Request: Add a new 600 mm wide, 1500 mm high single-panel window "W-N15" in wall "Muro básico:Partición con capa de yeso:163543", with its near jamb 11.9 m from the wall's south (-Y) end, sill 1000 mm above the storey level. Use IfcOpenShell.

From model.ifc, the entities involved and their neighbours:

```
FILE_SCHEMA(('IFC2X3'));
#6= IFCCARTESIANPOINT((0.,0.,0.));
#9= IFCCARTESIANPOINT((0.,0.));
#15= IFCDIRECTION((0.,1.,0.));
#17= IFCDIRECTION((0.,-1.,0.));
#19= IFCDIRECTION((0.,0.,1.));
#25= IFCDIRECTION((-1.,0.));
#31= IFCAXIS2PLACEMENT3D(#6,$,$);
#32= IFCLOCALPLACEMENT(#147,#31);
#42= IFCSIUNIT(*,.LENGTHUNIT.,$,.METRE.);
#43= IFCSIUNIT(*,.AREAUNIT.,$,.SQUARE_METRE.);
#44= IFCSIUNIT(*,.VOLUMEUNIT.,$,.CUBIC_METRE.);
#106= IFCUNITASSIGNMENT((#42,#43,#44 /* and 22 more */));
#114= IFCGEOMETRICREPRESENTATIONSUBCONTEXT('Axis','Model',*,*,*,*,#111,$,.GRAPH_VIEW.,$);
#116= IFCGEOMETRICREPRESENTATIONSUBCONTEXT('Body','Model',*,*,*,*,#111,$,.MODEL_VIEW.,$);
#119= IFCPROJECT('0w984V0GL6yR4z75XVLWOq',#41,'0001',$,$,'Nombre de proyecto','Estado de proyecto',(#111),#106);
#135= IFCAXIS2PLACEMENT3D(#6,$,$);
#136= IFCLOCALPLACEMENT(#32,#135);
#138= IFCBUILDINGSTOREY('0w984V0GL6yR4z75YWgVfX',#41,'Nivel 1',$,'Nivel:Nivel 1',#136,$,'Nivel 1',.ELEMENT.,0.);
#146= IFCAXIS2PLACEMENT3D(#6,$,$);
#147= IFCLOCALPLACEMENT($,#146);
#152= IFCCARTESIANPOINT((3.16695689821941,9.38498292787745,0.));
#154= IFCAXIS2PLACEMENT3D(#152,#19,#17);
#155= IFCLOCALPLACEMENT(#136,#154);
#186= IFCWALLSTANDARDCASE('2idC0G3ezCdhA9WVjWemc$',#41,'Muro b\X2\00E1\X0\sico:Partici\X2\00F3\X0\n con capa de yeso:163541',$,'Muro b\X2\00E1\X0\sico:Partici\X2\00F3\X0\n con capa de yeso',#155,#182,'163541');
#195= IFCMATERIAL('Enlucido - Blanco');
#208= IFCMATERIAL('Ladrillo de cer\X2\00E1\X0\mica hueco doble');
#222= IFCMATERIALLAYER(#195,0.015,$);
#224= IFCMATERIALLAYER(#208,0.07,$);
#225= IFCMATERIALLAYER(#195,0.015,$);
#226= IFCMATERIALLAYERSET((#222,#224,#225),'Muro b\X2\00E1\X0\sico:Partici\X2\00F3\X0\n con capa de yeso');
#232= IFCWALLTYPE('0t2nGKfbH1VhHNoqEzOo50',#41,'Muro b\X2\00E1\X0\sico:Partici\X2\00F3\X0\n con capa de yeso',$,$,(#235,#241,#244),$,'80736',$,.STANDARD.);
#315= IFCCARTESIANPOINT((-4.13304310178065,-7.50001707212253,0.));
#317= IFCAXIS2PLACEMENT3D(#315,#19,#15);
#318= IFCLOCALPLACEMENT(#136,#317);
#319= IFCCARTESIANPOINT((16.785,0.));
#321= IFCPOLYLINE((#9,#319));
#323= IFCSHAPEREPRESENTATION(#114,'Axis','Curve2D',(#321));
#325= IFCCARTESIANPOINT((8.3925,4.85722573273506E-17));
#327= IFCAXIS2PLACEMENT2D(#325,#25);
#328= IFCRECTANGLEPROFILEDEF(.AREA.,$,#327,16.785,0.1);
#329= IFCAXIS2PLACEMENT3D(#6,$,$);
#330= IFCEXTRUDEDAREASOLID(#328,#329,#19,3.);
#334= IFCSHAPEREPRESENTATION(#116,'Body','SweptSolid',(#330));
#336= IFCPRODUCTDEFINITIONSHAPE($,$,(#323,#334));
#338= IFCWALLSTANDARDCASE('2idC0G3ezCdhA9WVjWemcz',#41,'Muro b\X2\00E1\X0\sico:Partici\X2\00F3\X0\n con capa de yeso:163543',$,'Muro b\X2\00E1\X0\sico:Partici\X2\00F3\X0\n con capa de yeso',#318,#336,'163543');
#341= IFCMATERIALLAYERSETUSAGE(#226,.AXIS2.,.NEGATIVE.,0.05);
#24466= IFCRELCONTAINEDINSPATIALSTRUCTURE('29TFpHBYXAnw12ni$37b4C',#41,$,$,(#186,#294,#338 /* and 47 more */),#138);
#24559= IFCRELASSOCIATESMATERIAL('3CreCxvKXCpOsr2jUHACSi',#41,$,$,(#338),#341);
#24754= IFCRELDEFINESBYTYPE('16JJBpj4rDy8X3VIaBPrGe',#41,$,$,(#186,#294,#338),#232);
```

```python
import numpy as np
import ifcopenshell
import ifcopenshell.api.feature
import ifcopenshell.api.geometry
import ifcopenshell.api.root
import ifcopenshell.api.spatial
import ifcopenshell.api.type
import ifcopenshell.geom
import ifcopenshell.util.element
import ifcopenshell.util.placement
import ifcopenshell.util.representation
import ifcopenshell.util.shape
import ifcopenshell.util.unit

model = ifcopenshell.open("model.ifc")
unit_scale = ifcopenshell.util.unit.calculate_unit_scale(model)
settings = ifcopenshell.geom.settings()


def volume(element):
    """Net volume in cubic metres, openings subtracted."""
    shape = ifcopenshell.geom.create_shape(settings, element)
    return ifcopenshell.util.shape.get_volume(shape.geometry)


wall = model.by_guid("2idC0G3ezCdhA9WVjWemcz")
storey = ifcopenshell.util.element.get_container(wall, ifc_class="IfcBuildingStorey")
context = ifcopenshell.util.representation.get_context(model, "Model", "Body", "MODEL_VIEW")
before = volume(wall)

width, height, from_end, sill = 0.6, 1.5, 11.9, 1  # metres

# The wall runs along its own X axis, and the end named is its -X end.
wall_shape = ifcopenshell.geom.create_shape(settings, wall)
x, y, z = ifcopenshell.util.shape.get_vertices(wall_shape.geometry).T
start = x.min() + from_end
face, thickness = float(y.min()), float(y.max() - y.min())
wall_matrix = ifcopenshell.util.placement.get_local_placement(wall.ObjectPlacement)
level = ifcopenshell.util.placement.get_local_placement(storey.ObjectPlacement)[2, 3]


def in_wall(x, y):
    """Placement at x, y metres in the wall's axes, at sill height."""
    matrix = wall_matrix.copy()
    matrix[:, 3] = wall_matrix @ np.array([x / unit_scale, y / unit_scale, 0.0, 1.0])
    matrix[2, 3] = level + sill / unit_scale
    return matrix


# Opening: a box that overshoots both wall faces by 50 mm.
opening = ifcopenshell.api.root.create_entity(model, ifc_class="IfcOpeningElement")
box = ifcopenshell.api.geometry.add_wall_representation(
    model, context=context, length=width, height=height, thickness=thickness + 0.1
)
ifcopenshell.api.geometry.assign_representation(model, product=opening, representation=box)
ifcopenshell.api.geometry.edit_object_placement(model, product=opening, matrix=in_wall(start, face - 0.05), is_si=False)
ifcopenshell.api.feature.add_feature(model, feature=opening, element=wall)

window = ifcopenshell.api.root.create_entity(model, ifc_class="IfcWindow", name="W-N15")
window.OverallWidth, window.OverallHeight = width / unit_scale, height / unit_scale
body = ifcopenshell.api.geometry.add_window_representation(
    model,
    context=context,
    overall_width=window.OverallWidth,
    overall_height=window.OverallHeight,
    partition_type="SINGLE_PANEL",
)
ifcopenshell.api.geometry.assign_representation(model, product=window, representation=body)
ifcopenshell.api.spatial.assign_container(model, products=[window], relating_structure=storey)
fills = ifcopenshell.api.feature.add_filling(model, opening=opening, element=window)
fills.OwnerHistory = window.OwnerHistory  # required in IFC2X3

# IFC2X3 keeps the operation on the window style.
style = ifcopenshell.api.root.create_entity(model, ifc_class="IfcWindowStyle", name="W-N15")
style.OperationType, style.ConstructionType = "SINGLE_PANEL", "NOTDEFINED"
style.ParameterTakesPrecedence = style.Sizeable = False
ifcopenshell.api.type.assign_type(model, related_objects=[window], relating_type=style)

# Centre the window in the wall's thickness.
ifcopenshell.api.geometry.edit_object_placement(model, product=window, matrix=in_wall(start, face), is_si=False)
window_shape = ifcopenshell.geom.create_shape(settings, window)
depth = ifcopenshell.util.shape.get_vertices(window_shape.geometry)[:, 1]
offset = face + thickness / 2 - (depth.min() + depth.max()) / 2
ifcopenshell.api.geometry.edit_object_placement(model, product=window, matrix=in_wall(start, offset), is_si=False)

after = volume(wall)

print(f"wall volume {before:.3f} -> {after:.3f} m3")

model.write("model_edited.ifc")
```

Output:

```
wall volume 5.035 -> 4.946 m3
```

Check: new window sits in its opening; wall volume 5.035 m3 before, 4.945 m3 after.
